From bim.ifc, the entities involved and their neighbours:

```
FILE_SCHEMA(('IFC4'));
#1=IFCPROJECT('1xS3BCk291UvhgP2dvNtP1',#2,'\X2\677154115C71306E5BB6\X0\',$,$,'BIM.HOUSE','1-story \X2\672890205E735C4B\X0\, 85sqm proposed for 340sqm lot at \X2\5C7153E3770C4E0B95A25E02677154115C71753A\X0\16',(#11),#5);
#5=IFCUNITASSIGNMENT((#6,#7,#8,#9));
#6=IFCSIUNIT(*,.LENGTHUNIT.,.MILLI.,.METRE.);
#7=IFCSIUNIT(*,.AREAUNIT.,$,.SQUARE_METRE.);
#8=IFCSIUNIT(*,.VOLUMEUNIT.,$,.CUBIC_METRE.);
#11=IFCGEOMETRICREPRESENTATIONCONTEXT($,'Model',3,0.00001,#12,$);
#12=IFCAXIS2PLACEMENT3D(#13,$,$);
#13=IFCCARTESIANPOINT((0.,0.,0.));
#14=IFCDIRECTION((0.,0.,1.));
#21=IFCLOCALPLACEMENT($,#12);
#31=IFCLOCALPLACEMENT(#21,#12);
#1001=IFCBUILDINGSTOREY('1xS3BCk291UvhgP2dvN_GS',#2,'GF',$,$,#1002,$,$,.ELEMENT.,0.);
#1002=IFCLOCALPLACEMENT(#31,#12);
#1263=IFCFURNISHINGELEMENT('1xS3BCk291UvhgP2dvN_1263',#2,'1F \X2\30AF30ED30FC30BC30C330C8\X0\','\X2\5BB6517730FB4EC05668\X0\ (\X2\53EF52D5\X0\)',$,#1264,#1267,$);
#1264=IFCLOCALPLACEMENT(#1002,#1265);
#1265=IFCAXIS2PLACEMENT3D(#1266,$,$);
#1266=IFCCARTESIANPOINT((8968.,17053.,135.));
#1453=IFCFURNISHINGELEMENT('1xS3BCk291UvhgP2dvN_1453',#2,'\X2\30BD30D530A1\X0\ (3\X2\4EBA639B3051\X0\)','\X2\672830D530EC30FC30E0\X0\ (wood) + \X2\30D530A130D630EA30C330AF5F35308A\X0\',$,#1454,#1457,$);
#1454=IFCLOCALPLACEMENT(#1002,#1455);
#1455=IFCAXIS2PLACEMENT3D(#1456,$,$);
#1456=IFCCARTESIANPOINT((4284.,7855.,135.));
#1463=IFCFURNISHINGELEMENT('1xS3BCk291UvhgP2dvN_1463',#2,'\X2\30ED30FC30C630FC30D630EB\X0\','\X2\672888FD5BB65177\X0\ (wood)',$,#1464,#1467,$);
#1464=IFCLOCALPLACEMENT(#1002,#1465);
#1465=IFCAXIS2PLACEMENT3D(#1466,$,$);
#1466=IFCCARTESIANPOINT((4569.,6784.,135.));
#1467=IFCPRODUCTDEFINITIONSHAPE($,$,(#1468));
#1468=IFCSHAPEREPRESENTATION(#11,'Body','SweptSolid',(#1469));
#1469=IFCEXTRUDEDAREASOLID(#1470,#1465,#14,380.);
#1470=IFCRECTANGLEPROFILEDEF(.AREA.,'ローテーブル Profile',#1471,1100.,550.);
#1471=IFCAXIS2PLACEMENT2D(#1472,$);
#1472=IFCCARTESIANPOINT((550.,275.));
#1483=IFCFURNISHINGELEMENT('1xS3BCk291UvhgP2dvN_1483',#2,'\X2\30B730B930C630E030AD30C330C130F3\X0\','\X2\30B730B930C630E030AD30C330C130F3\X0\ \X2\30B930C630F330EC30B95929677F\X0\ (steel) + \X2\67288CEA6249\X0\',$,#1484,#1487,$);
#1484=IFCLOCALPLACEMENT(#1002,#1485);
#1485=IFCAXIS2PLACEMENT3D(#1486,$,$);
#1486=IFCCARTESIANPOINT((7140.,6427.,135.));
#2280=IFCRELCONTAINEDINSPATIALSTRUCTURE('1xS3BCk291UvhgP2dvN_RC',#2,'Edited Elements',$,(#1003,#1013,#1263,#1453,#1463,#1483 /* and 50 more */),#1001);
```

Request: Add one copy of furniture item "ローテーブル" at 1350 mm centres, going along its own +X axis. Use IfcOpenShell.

```python
import ifcopenshell
import ifcopenshell.api.geometry
import ifcopenshell.api.root
import ifcopenshell.util.element
import ifcopenshell.util.placement
import ifcopenshell.util.unit

model = ifcopenshell.open("bim.ifc")
unit_scale = ifcopenshell.util.unit.calculate_unit_scale(model)


def reuse_history(source, copy):
    """copy_class also copies each property set's owner history, people and application; keep the originals."""
    for rel in copy.IsDefinedBy:
        if rel.is_a("IfcRelDefinesByProperties") and (history := rel.RelatingPropertyDefinition.OwnerHistory):
            rel.RelatingPropertyDefinition.OwnerHistory = source.OwnerHistory
            ifcopenshell.util.element.remove_deep2(model, history)


source = model.by_guid("1xS3BCk291UvhgP2dvN_1463")
base = ifcopenshell.util.placement.get_local_placement(source.ObjectPlacement)
step = base[:3, 0] * 1.35 / unit_scale

for i in range(1, 2):
    copy = ifcopenshell.api.root.copy_class(model, product=source)
    copy.Representation = ifcopenshell.util.element.copy_deep(
        model, source.Representation, exclude=["IfcGeometricRepresentationContext", "IfcRepresentationMap"]
    )
    reuse_history(source, copy)
    matrix = base.copy()
    matrix[:3, 3] += i * step
    print("added at", matrix[:3, 3].round(3) + 0.0)
    ifcopenshell.api.geometry.edit_object_placement(model, product=copy, matrix=matrix, is_si=False)

model.write("bim_edited.ifc")
```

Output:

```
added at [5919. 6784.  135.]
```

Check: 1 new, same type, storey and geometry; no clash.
